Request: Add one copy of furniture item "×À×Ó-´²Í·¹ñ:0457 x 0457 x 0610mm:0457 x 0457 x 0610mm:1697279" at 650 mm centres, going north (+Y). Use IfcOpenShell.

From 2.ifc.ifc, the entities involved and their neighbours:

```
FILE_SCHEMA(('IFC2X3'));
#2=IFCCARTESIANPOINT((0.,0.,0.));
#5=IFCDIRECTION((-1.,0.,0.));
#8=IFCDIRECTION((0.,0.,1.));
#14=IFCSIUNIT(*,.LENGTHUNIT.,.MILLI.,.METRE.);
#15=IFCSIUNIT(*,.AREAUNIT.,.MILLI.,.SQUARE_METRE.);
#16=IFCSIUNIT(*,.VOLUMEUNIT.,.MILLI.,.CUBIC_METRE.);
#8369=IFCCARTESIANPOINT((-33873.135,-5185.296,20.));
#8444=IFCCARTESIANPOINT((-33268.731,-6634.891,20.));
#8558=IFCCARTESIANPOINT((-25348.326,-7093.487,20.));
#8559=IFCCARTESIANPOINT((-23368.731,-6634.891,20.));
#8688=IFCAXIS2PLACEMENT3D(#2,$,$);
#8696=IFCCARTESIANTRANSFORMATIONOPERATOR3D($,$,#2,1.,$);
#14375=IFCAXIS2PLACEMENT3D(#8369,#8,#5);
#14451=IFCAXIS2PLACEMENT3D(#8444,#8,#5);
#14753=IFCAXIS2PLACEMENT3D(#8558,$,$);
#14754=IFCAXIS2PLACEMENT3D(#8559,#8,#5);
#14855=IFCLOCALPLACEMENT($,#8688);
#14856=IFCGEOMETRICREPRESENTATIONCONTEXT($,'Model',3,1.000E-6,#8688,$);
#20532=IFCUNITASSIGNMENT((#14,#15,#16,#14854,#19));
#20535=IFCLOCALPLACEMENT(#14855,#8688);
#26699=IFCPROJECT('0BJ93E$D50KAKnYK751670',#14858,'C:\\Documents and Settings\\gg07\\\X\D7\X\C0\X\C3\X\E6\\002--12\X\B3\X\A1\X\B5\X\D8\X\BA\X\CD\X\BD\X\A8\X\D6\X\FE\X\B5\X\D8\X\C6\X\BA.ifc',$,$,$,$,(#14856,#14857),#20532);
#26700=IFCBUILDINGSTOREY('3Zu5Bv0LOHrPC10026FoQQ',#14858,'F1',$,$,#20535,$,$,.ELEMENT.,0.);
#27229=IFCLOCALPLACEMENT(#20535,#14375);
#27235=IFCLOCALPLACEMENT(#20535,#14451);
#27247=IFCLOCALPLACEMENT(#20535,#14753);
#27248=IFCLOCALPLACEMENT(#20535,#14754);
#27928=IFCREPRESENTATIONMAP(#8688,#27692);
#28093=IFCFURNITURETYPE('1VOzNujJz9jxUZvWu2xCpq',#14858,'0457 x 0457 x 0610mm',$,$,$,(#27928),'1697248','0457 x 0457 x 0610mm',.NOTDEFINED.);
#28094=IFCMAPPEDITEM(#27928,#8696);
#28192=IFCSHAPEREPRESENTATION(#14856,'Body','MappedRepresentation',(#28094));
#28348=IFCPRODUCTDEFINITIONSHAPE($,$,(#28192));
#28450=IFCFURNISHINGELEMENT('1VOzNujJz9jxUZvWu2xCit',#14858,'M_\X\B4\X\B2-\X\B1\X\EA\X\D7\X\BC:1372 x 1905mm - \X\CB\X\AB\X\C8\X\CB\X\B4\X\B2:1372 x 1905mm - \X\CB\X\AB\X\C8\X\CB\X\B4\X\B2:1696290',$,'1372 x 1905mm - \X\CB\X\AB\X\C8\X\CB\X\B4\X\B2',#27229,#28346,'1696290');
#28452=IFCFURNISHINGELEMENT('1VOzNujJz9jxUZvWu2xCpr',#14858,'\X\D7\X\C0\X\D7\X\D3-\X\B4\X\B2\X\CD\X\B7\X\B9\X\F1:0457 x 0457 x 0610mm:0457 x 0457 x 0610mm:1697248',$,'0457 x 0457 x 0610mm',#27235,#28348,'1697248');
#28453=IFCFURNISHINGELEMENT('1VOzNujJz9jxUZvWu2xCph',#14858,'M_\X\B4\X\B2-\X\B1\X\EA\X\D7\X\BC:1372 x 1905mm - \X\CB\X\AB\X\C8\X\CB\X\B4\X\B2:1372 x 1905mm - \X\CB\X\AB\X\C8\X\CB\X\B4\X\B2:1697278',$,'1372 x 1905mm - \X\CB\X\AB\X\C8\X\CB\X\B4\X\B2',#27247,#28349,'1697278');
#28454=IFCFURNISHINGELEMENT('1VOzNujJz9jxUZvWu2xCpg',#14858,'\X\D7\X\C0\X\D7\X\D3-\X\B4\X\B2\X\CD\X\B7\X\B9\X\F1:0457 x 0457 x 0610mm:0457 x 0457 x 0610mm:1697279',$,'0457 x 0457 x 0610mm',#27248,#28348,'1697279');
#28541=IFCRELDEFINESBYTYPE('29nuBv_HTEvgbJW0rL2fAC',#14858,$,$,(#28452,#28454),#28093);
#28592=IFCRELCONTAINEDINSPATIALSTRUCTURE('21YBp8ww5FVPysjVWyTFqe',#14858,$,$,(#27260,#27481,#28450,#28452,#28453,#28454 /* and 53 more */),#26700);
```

```python
import numpy as np
import ifcopenshell
import ifcopenshell.api.geometry
import ifcopenshell.api.root
import ifcopenshell.util.element
import ifcopenshell.util.placement

model = ifcopenshell.open("2.ifc.ifc")


def reuse_history(source, copy):
    """copy_class also copies each property set's owner history, people and application; keep the originals."""
    for rel in copy.IsDefinedBy:
        if rel.is_a("IfcRelDefinesByProperties") and (history := rel.RelatingPropertyDefinition.OwnerHistory):
            rel.RelatingPropertyDefinition.OwnerHistory = source.OwnerHistory
            ifcopenshell.util.element.remove_deep2(model, history)


source = model.by_guid("1VOzNujJz9jxUZvWu2xCpg")
base = ifcopenshell.util.placement.get_local_placement(source.ObjectPlacement)
step = np.array([0.0, 1.0, 0.0]) * 650.0

for i in range(1, 2):
    copy = ifcopenshell.api.root.copy_class(model, product=source)
    copy.Representation = ifcopenshell.util.element.copy_deep(
        model, source.Representation, exclude=["IfcGeometricRepresentationContext", "IfcRepresentationMap"]
    )
    copy.Name = "×À×Ó-´²Í·¹ñ:0457 x 0457 x 0610mm:0457 x 0457 x 0610mm"
    copy.Tag = None
    reuse_history(source, copy)
    matrix = base.copy()
    matrix[:3, 3] += i * step
    print("added at", matrix[:3, 3].round(3) + 0.0)
    ifcopenshell.api.geometry.edit_object_placement(model, product=copy, matrix=matrix, is_si=False)

model.write("2.ifc_v2.ifc")
```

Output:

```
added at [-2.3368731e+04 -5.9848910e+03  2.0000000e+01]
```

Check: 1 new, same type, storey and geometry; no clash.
